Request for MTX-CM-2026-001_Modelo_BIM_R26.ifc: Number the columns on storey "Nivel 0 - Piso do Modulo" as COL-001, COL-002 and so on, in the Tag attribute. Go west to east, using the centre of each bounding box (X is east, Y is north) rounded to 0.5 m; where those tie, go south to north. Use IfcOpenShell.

First a look at what the model holds.

```python
import ifcopenshell
import ifcopenshell.util.element
import ifcopenshell.util.placement

model = ifcopenshell.open("MTX-CM-2026-001_Modelo_BIM_R26.ifc")
print(model.schema)
storey = next(s for s in model.by_type("IfcBuildingStorey") if s.Name == "Nivel 0 - Piso do Modulo")
columns = [e for e in ifcopenshell.util.element.get_decomposition(storey) if e.is_a("IfcColumn")]
for e in sorted(columns, key=lambda e: e.id()):
    origin = ifcopenshell.util.placement.get_local_placement(e.ObjectPlacement)[:3, 3]
    print(e.id(), e.Tag, e.Name, origin.round(2) + 0.0, sep=" | ")
```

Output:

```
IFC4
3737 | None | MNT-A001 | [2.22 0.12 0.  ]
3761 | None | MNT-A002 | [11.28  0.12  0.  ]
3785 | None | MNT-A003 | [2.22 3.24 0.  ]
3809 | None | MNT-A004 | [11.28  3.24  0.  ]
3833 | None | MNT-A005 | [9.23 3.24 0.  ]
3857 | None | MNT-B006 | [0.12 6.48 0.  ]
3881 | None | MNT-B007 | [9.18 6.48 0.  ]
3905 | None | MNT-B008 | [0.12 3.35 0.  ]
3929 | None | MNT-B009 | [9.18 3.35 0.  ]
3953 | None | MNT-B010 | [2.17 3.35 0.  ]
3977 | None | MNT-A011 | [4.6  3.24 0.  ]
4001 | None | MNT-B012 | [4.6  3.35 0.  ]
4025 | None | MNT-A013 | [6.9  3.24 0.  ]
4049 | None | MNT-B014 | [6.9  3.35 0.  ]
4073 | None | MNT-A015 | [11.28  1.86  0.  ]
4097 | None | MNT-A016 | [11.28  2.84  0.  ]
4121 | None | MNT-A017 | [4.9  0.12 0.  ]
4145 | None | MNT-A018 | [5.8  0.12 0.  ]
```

```python
import ifcopenshell
import ifcopenshell.geom
import ifcopenshell.util.element
import ifcopenshell.util.shape

model = ifcopenshell.open("MTX-CM-2026-001_Modelo_BIM_R26.ifc")
settings = ifcopenshell.geom.settings()
settings.set("use-world-coords", True)


def centre(element):
    shape = ifcopenshell.geom.create_shape(settings, element)
    return ifcopenshell.util.shape.get_bbox_centroid(shape.geometry)


storey = next(s for s in model.by_type("IfcBuildingStorey") if s.Name == "Nivel 0 - Piso do Modulo")
columns = [e for e in ifcopenshell.util.element.get_decomposition(storey) if e.is_a("IfcColumn")]

# Insertion points can sit at a corner or the storey origin, so sort by the geometry (in metres).
centres = {e: centre(e) for e in columns}
columns.sort(key=lambda e: (round(centres[e][0] / 0.5), centres[e][1]))

for i, e in enumerate(columns, start=1):
    number = f"COL-0{i:02d}"
    e.Tag = number
    print(e.id(), number)

model.write("MTX-CM-2026-001_Modelo_BIM_R26_edited.ifc")
```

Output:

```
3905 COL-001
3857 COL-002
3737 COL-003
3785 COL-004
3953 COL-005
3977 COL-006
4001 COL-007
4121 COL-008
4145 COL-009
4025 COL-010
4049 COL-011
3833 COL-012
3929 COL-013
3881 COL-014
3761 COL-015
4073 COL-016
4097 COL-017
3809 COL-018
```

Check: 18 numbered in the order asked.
